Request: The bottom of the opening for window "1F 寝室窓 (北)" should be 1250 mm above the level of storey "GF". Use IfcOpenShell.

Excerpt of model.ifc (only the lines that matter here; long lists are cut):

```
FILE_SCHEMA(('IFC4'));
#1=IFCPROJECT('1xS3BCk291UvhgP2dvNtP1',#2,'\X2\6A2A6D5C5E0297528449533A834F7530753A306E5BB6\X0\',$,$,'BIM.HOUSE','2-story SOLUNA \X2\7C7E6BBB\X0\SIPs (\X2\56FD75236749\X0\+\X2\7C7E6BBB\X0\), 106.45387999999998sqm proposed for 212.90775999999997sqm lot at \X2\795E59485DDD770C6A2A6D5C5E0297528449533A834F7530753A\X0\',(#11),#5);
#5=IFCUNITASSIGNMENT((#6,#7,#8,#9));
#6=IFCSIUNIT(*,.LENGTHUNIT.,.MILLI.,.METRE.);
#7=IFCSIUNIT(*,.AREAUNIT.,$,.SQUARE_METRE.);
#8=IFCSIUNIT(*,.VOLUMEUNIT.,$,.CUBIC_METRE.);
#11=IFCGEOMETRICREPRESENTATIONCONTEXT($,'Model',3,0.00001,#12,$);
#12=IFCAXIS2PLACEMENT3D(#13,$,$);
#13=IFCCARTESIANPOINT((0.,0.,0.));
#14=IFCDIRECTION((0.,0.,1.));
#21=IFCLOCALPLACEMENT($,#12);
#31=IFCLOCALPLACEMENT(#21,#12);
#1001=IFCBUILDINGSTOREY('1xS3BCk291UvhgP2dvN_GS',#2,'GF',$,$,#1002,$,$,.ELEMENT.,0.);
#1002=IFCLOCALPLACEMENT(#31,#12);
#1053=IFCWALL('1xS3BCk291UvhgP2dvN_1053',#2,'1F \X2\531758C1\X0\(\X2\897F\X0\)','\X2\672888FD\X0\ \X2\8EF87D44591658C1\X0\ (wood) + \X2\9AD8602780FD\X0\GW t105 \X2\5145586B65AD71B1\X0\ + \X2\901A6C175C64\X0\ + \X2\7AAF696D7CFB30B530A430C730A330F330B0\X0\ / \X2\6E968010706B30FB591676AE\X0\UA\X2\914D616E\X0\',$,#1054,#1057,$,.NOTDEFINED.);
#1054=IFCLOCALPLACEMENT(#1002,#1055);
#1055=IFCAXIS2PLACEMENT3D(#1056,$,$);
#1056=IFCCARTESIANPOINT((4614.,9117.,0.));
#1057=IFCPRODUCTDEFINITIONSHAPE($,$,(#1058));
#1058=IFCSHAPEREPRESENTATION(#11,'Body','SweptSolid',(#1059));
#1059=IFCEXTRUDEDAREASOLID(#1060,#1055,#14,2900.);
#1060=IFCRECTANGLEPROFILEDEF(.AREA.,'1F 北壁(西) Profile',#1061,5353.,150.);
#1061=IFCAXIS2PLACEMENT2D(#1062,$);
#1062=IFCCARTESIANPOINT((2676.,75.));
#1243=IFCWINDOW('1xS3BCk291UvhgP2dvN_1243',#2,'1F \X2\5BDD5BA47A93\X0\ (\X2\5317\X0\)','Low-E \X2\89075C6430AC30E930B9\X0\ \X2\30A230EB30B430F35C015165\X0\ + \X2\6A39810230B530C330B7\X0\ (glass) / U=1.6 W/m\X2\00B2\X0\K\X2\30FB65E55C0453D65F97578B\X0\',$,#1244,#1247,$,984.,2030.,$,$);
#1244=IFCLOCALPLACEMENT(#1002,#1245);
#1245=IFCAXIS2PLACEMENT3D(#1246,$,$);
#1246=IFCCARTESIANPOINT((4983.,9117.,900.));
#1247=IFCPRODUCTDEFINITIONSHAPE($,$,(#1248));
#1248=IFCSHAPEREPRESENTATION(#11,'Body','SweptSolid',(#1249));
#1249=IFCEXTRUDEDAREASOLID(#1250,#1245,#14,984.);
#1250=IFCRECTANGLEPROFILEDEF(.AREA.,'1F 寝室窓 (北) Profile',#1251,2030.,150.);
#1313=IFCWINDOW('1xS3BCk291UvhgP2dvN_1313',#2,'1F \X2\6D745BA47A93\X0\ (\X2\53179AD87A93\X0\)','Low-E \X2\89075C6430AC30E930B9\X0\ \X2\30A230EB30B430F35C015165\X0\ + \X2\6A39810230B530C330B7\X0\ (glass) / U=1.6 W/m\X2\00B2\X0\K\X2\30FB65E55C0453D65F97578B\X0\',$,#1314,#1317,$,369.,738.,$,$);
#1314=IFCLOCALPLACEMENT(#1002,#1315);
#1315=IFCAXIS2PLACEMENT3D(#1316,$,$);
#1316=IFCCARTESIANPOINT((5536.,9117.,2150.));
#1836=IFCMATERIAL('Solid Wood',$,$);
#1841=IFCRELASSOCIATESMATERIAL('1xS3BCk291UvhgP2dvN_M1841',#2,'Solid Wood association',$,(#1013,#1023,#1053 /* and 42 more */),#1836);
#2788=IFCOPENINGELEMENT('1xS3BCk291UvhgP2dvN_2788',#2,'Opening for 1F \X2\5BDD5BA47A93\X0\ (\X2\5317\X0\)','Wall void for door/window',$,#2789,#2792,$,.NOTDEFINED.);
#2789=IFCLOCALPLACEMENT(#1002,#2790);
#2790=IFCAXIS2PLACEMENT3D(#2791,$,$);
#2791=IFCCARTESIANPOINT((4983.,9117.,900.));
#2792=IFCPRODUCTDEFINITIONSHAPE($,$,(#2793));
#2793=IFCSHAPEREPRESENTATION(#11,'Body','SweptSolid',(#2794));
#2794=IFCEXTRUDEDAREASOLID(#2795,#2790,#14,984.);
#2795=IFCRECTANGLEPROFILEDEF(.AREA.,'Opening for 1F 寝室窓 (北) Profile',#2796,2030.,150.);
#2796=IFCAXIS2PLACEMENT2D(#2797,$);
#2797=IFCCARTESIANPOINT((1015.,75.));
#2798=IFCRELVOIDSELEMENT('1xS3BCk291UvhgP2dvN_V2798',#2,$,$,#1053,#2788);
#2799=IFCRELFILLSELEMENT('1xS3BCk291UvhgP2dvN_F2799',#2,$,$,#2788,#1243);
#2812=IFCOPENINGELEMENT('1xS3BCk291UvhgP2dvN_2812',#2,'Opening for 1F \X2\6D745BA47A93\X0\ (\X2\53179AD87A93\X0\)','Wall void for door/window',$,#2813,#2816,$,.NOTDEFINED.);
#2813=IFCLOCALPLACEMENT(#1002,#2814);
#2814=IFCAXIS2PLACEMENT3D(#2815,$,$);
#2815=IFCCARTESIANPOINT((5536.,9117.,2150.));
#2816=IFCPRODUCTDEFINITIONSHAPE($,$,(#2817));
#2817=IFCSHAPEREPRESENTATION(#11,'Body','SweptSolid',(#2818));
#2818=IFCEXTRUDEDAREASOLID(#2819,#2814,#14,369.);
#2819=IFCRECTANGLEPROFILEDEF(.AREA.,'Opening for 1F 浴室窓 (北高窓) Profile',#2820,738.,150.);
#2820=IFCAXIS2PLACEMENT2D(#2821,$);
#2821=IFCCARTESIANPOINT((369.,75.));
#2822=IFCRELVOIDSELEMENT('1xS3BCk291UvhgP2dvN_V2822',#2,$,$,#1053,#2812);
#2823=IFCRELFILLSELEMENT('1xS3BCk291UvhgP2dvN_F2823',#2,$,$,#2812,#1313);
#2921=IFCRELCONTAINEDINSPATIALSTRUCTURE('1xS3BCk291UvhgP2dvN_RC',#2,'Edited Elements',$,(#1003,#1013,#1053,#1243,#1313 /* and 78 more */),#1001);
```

```python
import numpy as np
import ifcopenshell
import ifcopenshell.api.geometry
import ifcopenshell.geom
import ifcopenshell.util.element
import ifcopenshell.util.placement
import ifcopenshell.util.shape
import ifcopenshell.util.unit

model = ifcopenshell.open("model.ifc")
unit_scale = ifcopenshell.util.unit.calculate_unit_scale(model)

window = model.by_guid("1xS3BCk291UvhgP2dvN_1243")
opening = window.FillsVoids[0].RelatingOpeningElement
storey = ifcopenshell.util.element.get_container(window, ifc_class="IfcBuildingStorey")
level = ifcopenshell.util.placement.get_local_placement(storey.ObjectPlacement)[2, 3]

# The opening's origin need not be at the sill, so measure its lowest point.
shape = ifcopenshell.geom.create_shape(ifcopenshell.geom.settings(), opening)
bottom = ifcopenshell.util.shape.get_shape_bottom_elevation(shape, shape.geometry) / unit_scale
dz = level + 1.25 / unit_scale - bottom

shift = np.array([0.0, 0.0, dz])
# The window is not placed relative to its opening, so move both.
for product in (opening, window):
    matrix = ifcopenshell.util.placement.get_local_placement(product.ObjectPlacement)
    matrix[:3, 3] += shift
    ifcopenshell.api.geometry.edit_object_placement(model, product=product, matrix=matrix, is_si=False)

print(f"moved by {dz * unit_scale:+.3f} m")

model.write("model-out.ifc")
```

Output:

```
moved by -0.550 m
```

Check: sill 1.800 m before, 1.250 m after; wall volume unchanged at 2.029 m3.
